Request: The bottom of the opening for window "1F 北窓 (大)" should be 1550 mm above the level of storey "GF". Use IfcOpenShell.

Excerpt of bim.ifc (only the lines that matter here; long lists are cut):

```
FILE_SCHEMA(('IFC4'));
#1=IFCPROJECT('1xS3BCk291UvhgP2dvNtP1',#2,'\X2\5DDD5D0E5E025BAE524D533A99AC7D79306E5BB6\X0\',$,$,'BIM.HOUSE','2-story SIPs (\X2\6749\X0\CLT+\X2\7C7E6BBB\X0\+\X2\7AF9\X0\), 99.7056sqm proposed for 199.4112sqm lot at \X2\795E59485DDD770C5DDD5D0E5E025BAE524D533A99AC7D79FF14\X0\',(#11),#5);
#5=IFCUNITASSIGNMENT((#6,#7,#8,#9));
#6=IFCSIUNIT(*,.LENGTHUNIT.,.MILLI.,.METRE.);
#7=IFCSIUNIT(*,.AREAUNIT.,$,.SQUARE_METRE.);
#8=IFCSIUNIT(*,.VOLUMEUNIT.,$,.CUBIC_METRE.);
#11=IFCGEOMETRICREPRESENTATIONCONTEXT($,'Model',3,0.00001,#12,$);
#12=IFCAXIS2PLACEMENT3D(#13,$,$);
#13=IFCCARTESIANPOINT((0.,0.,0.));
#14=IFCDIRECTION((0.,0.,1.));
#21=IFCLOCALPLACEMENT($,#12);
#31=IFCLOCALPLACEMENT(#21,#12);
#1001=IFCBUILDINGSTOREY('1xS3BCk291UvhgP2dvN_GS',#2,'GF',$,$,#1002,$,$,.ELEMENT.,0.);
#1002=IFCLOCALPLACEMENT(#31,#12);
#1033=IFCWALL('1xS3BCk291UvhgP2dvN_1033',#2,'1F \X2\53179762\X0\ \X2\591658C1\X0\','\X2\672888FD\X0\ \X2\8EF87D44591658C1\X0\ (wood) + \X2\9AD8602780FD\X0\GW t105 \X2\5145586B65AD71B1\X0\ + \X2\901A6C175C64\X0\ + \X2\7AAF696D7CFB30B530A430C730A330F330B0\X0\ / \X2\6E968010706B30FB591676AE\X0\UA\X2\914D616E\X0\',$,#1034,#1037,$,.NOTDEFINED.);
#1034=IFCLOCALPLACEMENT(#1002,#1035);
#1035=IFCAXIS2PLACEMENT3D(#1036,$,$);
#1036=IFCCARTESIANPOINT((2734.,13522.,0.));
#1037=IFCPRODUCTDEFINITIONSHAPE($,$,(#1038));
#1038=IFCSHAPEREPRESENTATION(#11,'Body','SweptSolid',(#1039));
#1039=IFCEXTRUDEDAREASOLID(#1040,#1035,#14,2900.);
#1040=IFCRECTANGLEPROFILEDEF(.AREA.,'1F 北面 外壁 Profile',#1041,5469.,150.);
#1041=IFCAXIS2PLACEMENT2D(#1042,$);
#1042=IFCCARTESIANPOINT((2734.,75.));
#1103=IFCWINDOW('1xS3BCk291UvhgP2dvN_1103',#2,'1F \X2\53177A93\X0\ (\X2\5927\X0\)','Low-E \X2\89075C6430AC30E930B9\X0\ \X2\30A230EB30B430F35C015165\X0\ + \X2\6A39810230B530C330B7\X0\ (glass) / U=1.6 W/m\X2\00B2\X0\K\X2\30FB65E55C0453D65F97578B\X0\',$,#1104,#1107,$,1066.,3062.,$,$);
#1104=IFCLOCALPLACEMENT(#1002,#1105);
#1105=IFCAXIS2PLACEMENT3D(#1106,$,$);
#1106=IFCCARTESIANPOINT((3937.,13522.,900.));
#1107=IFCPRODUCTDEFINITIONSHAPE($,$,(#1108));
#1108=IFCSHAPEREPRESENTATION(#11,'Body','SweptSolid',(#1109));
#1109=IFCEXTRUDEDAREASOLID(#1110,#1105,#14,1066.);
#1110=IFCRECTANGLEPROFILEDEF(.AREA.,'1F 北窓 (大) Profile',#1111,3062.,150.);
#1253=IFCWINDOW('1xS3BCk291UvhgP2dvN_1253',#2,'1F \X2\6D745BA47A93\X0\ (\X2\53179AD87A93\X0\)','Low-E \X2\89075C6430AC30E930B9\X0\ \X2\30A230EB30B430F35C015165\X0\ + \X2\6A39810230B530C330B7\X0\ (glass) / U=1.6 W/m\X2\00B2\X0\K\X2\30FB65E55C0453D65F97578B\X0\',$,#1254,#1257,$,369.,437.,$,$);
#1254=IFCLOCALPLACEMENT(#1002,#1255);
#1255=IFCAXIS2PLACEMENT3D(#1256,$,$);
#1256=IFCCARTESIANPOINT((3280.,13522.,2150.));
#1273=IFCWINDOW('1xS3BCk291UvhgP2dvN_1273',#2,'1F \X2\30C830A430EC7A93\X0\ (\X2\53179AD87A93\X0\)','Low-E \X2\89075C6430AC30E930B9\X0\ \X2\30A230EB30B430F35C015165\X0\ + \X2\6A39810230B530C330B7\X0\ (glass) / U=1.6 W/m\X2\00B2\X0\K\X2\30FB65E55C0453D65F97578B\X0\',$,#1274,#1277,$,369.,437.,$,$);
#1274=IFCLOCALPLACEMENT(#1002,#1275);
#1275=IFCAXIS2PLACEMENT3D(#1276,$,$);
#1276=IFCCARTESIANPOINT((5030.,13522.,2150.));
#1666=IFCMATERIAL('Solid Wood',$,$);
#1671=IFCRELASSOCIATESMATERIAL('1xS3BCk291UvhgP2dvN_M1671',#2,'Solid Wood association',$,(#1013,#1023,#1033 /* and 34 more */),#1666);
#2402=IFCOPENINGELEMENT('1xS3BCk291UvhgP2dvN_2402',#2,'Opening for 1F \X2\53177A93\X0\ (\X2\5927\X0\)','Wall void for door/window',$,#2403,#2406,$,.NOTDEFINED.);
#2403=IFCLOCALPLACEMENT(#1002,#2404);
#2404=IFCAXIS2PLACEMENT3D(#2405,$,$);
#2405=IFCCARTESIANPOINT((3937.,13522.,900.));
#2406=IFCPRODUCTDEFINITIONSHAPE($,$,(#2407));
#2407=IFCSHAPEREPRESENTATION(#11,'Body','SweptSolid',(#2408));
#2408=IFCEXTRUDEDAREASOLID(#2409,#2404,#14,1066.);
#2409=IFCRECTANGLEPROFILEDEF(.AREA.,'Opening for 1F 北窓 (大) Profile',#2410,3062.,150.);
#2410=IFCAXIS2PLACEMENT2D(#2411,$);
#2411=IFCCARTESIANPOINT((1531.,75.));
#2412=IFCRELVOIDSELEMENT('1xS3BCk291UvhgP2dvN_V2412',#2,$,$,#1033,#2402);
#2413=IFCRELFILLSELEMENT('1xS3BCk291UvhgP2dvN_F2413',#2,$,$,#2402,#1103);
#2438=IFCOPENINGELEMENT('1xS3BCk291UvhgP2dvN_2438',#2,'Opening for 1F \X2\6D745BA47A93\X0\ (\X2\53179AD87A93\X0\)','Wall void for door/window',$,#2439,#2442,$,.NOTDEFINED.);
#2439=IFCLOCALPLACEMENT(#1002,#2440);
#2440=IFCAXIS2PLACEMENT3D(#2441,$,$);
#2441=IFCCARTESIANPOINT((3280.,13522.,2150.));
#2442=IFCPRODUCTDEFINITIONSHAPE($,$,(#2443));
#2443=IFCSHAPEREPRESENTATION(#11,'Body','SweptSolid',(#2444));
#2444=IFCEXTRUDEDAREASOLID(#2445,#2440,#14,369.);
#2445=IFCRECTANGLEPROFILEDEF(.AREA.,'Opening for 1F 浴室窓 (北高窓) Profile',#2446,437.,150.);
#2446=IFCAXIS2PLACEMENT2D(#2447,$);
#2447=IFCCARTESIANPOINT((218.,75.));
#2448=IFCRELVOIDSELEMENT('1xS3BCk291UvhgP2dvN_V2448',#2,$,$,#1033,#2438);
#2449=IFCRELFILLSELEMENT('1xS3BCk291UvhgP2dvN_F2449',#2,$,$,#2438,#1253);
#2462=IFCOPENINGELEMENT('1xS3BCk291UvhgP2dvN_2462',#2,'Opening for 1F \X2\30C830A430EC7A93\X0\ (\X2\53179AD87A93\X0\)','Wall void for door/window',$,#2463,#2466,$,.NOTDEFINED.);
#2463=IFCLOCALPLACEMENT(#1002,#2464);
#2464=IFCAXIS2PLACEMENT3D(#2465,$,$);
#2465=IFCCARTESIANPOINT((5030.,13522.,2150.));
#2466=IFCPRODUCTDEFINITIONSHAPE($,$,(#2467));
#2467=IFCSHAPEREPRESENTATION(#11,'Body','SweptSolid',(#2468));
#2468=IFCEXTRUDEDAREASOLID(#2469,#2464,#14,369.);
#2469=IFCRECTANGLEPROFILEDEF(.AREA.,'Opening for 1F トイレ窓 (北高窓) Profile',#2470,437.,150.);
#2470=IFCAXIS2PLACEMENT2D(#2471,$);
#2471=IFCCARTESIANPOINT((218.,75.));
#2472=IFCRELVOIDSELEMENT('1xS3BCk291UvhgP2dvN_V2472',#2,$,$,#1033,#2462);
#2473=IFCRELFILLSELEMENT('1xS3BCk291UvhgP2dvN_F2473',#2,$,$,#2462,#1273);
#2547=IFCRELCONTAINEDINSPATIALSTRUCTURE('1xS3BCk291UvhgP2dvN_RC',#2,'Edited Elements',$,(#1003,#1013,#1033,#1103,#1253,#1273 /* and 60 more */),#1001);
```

```python
import numpy as np
import ifcopenshell
import ifcopenshell.api.geometry
import ifcopenshell.geom
import ifcopenshell.util.element
import ifcopenshell.util.placement
import ifcopenshell.util.shape
import ifcopenshell.util.unit

model = ifcopenshell.open("bim.ifc")
unit_scale = ifcopenshell.util.unit.calculate_unit_scale(model)

window = model.by_guid("1xS3BCk291UvhgP2dvN_1103")
opening = window.FillsVoids[0].RelatingOpeningElement
storey = ifcopenshell.util.element.get_container(window, ifc_class="IfcBuildingStorey")
level = ifcopenshell.util.placement.get_local_placement(storey.ObjectPlacement)[2, 3]

# The opening's origin need not be at the sill, so measure its lowest point.
shape = ifcopenshell.geom.create_shape(ifcopenshell.geom.settings(), opening)
bottom = ifcopenshell.util.shape.get_shape_bottom_elevation(shape, shape.geometry) / unit_scale
dz = level + 1550.0 - bottom

shift = np.array([0.0, 0.0, dz])
# The window is not placed relative to its opening, so move both.
for product in (opening, window):
    matrix = ifcopenshell.util.placement.get_local_placement(product.ObjectPlacement)
    matrix[:3, 3] += shift
    ifcopenshell.api.geometry.edit_object_placement(model, product=product, matrix=matrix, is_si=False)

print(f"moved by {dz * unit_scale:+.3f} m")

model.write("bim_edited.ifc")
```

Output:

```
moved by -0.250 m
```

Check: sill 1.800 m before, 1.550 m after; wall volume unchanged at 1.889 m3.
